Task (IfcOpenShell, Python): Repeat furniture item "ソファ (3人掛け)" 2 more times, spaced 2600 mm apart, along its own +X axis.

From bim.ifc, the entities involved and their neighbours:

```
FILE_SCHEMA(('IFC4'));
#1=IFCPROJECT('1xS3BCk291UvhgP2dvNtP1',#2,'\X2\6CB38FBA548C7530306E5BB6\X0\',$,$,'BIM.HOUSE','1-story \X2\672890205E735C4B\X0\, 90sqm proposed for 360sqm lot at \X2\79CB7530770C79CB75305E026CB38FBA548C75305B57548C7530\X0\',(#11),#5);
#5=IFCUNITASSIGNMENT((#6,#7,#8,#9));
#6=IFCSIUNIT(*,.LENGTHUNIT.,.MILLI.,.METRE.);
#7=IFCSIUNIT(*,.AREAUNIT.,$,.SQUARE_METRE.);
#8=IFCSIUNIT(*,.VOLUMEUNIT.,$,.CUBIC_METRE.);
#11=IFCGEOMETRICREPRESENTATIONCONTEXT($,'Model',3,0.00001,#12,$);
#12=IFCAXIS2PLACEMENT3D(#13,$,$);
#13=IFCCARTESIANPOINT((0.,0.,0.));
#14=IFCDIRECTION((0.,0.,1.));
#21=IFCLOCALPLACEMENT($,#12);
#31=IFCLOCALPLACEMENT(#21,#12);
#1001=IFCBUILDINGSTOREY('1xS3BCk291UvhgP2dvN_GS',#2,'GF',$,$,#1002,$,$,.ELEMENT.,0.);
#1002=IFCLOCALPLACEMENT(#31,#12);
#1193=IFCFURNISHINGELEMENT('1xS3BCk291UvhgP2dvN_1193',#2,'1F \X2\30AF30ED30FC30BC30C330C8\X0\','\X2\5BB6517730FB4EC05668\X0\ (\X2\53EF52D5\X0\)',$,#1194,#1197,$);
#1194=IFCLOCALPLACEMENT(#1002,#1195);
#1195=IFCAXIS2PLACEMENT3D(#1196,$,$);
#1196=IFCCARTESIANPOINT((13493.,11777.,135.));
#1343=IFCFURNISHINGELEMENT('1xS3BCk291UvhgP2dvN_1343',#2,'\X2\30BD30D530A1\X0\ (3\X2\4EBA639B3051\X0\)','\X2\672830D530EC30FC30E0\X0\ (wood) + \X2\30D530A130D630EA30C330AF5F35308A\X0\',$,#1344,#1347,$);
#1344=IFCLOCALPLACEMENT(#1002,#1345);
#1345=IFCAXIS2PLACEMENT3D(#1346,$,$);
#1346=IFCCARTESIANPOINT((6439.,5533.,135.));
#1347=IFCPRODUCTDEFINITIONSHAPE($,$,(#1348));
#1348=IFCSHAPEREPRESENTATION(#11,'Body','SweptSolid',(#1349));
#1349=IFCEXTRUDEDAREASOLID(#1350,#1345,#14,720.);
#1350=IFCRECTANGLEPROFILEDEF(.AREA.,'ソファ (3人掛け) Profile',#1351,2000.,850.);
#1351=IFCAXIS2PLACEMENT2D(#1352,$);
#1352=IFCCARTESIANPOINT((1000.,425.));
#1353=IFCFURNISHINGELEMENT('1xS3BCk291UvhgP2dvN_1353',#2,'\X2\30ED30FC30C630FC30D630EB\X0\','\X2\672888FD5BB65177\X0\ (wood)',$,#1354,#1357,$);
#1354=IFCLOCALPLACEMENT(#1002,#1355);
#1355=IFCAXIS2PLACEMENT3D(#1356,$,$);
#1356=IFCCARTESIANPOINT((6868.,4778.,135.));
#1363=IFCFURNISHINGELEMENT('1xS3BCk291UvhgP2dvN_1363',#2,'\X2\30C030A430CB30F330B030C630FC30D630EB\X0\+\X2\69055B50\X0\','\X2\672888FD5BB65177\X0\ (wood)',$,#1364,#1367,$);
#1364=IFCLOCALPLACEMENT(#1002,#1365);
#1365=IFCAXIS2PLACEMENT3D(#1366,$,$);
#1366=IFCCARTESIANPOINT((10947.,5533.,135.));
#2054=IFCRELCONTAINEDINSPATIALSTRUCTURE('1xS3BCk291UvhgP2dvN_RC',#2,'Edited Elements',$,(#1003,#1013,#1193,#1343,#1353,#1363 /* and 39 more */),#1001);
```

```python
import ifcopenshell
import ifcopenshell.api.geometry
import ifcopenshell.api.root
import ifcopenshell.util.element
import ifcopenshell.util.placement
import ifcopenshell.util.unit

model = ifcopenshell.open("bim.ifc")
unit_scale = ifcopenshell.util.unit.calculate_unit_scale(model)


def reuse_history(source, copy):
    """copy_class also copies each property set's owner history, people and application; keep the originals."""
    for rel in copy.IsDefinedBy:
        if rel.is_a("IfcRelDefinesByProperties") and (history := rel.RelatingPropertyDefinition.OwnerHistory):
            rel.RelatingPropertyDefinition.OwnerHistory = source.OwnerHistory
            ifcopenshell.util.element.remove_deep2(model, history)


source = model.by_id(1343)
base = ifcopenshell.util.placement.get_local_placement(source.ObjectPlacement)
step = base[:3, 0] * 2.6 / unit_scale

for i in range(1, 3):
    copy = ifcopenshell.api.root.copy_class(model, product=source)
    copy.Representation = ifcopenshell.util.element.copy_deep(
        model, source.Representation, exclude=["IfcGeometricRepresentationContext", "IfcRepresentationMap"]
    )
    reuse_history(source, copy)
    matrix = base.copy()
    matrix[:3, 3] += i * step
    print("added at", matrix[:3, 3].round(3) + 0.0)
    ifcopenshell.api.geometry.edit_object_placement(model, product=copy, matrix=matrix, is_si=False)

model.write("bim_rev.ifc")
```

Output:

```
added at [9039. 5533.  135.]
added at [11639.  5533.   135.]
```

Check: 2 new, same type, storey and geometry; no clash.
